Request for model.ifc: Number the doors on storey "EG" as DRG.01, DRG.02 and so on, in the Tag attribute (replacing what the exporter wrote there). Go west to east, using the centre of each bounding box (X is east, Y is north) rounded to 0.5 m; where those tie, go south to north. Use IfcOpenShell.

First a look at what the model holds.

```python
import ifcopenshell
import ifcopenshell.util.element
import ifcopenshell.util.placement

model = ifcopenshell.open("model.ifc")
print(model.schema)
storey = next(s for s in model.by_type("IfcBuildingStorey") if s.Name == "EG")
doors = [e for e in ifcopenshell.util.element.get_decomposition(storey) if e.is_a("IfcDoor")]
for e in sorted(doors, key=lambda e: e.id()):
    origin = ifcopenshell.util.placement.get_local_placement(e.ObjectPlacement)[:3, 3]
    print(e.id(), e.Tag, e.Name, origin.round(2) + 0.0, sep=" | ")
```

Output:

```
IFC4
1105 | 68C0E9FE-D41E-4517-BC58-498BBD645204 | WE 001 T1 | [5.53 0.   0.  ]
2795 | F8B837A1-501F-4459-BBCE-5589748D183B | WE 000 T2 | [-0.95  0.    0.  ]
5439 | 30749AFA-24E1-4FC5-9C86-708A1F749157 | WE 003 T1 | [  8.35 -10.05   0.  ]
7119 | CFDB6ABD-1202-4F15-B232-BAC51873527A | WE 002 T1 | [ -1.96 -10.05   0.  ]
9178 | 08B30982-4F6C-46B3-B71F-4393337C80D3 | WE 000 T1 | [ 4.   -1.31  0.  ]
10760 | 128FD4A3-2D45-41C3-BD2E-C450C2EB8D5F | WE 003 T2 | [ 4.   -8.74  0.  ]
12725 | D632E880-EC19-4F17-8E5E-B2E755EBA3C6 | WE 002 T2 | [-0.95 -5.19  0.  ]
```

```python
import ifcopenshell
import ifcopenshell.geom
import ifcopenshell.util.element
import ifcopenshell.util.shape

model = ifcopenshell.open("model.ifc")
settings = ifcopenshell.geom.settings()
settings.set("use-world-coords", True)


def centre(element):
    shape = ifcopenshell.geom.create_shape(settings, element)
    return ifcopenshell.util.shape.get_bbox_centroid(shape.geometry)


storey = next(s for s in model.by_type("IfcBuildingStorey") if s.Name == "EG")
doors = [e for e in ifcopenshell.util.element.get_decomposition(storey) if e.is_a("IfcDoor")]

# Insertion points can sit at a corner or the storey origin, so sort by the geometry (in metres).
centres = {e: centre(e) for e in doors}
doors.sort(key=lambda e: (round(centres[e][0] / 0.5), centres[e][1]))

for i, e in enumerate(doors, start=1):
    number = f"DRG.{i:02d}"
    e.Tag = number
    print(e.id(), number)

model.write("model-out.ifc")
```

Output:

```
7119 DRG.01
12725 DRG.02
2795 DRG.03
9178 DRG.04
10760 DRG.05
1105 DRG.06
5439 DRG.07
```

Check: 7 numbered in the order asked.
